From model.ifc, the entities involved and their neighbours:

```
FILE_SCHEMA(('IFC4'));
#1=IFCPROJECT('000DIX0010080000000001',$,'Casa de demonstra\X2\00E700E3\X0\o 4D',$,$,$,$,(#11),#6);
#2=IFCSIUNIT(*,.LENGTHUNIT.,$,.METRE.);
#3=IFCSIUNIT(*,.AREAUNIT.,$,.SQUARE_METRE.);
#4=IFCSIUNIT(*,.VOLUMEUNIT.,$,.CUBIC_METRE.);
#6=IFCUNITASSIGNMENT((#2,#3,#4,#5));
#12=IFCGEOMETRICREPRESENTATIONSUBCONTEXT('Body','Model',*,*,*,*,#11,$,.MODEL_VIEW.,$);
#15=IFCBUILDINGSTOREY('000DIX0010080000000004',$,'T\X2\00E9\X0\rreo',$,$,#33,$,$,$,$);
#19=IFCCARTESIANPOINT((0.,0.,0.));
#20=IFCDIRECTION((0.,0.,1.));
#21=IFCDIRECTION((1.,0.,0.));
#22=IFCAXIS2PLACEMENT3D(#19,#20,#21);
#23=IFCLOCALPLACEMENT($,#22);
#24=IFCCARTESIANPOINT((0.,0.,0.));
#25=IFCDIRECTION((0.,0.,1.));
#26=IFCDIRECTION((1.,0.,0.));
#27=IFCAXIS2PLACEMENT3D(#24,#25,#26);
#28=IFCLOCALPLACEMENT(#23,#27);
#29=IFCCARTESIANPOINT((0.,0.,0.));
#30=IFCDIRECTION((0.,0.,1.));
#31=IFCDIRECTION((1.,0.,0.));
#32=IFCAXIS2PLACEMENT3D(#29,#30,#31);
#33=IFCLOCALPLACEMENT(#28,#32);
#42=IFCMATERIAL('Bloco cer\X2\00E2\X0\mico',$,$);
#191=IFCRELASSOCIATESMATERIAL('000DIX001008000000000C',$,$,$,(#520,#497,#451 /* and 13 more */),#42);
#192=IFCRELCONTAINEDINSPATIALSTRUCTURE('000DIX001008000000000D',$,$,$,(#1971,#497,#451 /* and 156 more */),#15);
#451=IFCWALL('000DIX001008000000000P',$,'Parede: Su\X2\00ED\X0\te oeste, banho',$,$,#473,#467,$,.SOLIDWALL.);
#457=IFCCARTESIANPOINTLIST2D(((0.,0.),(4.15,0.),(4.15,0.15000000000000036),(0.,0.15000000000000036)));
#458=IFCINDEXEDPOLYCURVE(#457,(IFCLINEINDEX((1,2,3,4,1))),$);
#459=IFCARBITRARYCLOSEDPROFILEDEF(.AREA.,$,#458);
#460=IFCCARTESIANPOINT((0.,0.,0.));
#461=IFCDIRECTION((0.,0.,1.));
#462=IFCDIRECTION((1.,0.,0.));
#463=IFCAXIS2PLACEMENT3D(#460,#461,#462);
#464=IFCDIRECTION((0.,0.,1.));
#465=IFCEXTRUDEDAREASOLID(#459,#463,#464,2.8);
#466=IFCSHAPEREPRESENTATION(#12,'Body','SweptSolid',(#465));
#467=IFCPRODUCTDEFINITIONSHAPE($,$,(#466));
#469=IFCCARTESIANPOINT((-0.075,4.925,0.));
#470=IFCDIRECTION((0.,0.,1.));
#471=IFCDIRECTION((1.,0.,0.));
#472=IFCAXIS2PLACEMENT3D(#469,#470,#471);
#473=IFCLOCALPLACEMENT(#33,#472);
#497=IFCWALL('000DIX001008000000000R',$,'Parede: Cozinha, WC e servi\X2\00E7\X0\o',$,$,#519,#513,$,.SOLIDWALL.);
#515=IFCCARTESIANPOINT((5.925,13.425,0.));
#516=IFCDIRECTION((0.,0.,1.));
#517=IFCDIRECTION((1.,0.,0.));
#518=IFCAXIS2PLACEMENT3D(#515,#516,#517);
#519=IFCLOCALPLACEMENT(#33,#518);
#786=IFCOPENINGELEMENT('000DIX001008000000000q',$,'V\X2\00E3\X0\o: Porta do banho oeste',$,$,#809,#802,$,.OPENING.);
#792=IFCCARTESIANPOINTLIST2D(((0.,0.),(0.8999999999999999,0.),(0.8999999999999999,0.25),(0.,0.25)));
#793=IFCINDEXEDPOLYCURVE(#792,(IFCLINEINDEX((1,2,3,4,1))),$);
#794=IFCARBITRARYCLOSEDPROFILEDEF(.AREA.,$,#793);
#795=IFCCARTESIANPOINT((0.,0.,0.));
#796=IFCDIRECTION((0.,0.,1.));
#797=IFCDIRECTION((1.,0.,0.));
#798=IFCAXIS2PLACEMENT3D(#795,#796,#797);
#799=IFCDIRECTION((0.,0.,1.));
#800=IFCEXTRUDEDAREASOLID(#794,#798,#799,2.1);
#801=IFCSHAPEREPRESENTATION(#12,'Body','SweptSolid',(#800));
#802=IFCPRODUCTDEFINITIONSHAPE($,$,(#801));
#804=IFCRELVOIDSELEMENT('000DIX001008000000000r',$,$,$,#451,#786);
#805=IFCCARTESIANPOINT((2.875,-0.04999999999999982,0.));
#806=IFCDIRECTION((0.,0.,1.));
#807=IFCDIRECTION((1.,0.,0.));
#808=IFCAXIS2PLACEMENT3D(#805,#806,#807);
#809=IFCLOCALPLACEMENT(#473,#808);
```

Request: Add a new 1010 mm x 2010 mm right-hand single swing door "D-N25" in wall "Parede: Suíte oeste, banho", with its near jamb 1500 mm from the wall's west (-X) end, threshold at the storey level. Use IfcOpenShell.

```python
import numpy as np
import ifcopenshell
import ifcopenshell.api.feature
import ifcopenshell.api.geometry
import ifcopenshell.api.root
import ifcopenshell.api.spatial
import ifcopenshell.geom
import ifcopenshell.util.element
import ifcopenshell.util.placement
import ifcopenshell.util.representation
import ifcopenshell.util.shape
import ifcopenshell.util.unit

model = ifcopenshell.open("model.ifc")
unit_scale = ifcopenshell.util.unit.calculate_unit_scale(model)
settings = ifcopenshell.geom.settings()


def volume(element):
    """Net volume in cubic metres, openings subtracted."""
    shape = ifcopenshell.geom.create_shape(settings, element)
    return ifcopenshell.util.shape.get_volume(shape.geometry)


wall = model.by_guid("000DIX001008000000000P")
storey = ifcopenshell.util.element.get_container(wall, ifc_class="IfcBuildingStorey")
context = ifcopenshell.util.representation.get_context(model, "Model", "Body", "MODEL_VIEW")
before = volume(wall)

width, height, from_end, sill = 1.01, 2.01, 1.5, 0.0  # metres

# The wall runs along its own X axis, and the end named is its -X end.
wall_shape = ifcopenshell.geom.create_shape(settings, wall)
x, y, z = ifcopenshell.util.shape.get_vertices(wall_shape.geometry).T
start = x.min() + from_end
face, thickness = float(y.min()), float(y.max() - y.min())
wall_matrix = ifcopenshell.util.placement.get_local_placement(wall.ObjectPlacement)
level = ifcopenshell.util.placement.get_local_placement(storey.ObjectPlacement)[2, 3]


def in_wall(x, y):
    """Placement at x, y metres in the wall's axes, at sill height."""
    matrix = wall_matrix.copy()
    matrix[:, 3] = wall_matrix @ np.array([x / unit_scale, y / unit_scale, 0.0, 1.0])
    matrix[2, 3] = level + sill / unit_scale
    return matrix


# Opening: a box that overshoots both wall faces by 50 mm.
opening = ifcopenshell.api.root.create_entity(model, ifc_class="IfcOpeningElement", predefined_type="OPENING")
box = ifcopenshell.api.geometry.add_wall_representation(
    model, context=context, length=width, height=height, thickness=thickness + 0.1
)
ifcopenshell.api.geometry.assign_representation(model, product=opening, representation=box)
ifcopenshell.api.geometry.edit_object_placement(model, product=opening, matrix=in_wall(start, face - 0.05), is_si=False)
ifcopenshell.api.feature.add_feature(model, feature=opening, element=wall)

door = ifcopenshell.api.root.create_entity(model, ifc_class="IfcDoor", name="D-N25", predefined_type="DOOR")
door.OverallWidth, door.OverallHeight = width / unit_scale, height / unit_scale
door.OperationType = "SINGLE_SWING_RIGHT"
body = ifcopenshell.api.geometry.add_door_representation(
    model,
    context=context,
    overall_width=door.OverallWidth,
    overall_height=door.OverallHeight,
    operation_type="SINGLE_SWING_RIGHT",
    lining_properties={"LiningDepth": thickness / unit_scale, "ThresholdDepth": thickness / unit_scale},
)
ifcopenshell.api.geometry.assign_representation(model, product=door, representation=body)
ifcopenshell.api.spatial.assign_container(model, products=[door], relating_structure=storey)
ifcopenshell.api.feature.add_filling(model, opening=opening, element=door)

# The lining spans the wall, so the door starts at the wall face.
ifcopenshell.api.geometry.edit_object_placement(model, product=door, matrix=in_wall(start, face), is_si=False)

after = volume(wall)

print(f"wall volume {before:.3f} -> {after:.3f} m3")

model.write("model_edited.ifc")
```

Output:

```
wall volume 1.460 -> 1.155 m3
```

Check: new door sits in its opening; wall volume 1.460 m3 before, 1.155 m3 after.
